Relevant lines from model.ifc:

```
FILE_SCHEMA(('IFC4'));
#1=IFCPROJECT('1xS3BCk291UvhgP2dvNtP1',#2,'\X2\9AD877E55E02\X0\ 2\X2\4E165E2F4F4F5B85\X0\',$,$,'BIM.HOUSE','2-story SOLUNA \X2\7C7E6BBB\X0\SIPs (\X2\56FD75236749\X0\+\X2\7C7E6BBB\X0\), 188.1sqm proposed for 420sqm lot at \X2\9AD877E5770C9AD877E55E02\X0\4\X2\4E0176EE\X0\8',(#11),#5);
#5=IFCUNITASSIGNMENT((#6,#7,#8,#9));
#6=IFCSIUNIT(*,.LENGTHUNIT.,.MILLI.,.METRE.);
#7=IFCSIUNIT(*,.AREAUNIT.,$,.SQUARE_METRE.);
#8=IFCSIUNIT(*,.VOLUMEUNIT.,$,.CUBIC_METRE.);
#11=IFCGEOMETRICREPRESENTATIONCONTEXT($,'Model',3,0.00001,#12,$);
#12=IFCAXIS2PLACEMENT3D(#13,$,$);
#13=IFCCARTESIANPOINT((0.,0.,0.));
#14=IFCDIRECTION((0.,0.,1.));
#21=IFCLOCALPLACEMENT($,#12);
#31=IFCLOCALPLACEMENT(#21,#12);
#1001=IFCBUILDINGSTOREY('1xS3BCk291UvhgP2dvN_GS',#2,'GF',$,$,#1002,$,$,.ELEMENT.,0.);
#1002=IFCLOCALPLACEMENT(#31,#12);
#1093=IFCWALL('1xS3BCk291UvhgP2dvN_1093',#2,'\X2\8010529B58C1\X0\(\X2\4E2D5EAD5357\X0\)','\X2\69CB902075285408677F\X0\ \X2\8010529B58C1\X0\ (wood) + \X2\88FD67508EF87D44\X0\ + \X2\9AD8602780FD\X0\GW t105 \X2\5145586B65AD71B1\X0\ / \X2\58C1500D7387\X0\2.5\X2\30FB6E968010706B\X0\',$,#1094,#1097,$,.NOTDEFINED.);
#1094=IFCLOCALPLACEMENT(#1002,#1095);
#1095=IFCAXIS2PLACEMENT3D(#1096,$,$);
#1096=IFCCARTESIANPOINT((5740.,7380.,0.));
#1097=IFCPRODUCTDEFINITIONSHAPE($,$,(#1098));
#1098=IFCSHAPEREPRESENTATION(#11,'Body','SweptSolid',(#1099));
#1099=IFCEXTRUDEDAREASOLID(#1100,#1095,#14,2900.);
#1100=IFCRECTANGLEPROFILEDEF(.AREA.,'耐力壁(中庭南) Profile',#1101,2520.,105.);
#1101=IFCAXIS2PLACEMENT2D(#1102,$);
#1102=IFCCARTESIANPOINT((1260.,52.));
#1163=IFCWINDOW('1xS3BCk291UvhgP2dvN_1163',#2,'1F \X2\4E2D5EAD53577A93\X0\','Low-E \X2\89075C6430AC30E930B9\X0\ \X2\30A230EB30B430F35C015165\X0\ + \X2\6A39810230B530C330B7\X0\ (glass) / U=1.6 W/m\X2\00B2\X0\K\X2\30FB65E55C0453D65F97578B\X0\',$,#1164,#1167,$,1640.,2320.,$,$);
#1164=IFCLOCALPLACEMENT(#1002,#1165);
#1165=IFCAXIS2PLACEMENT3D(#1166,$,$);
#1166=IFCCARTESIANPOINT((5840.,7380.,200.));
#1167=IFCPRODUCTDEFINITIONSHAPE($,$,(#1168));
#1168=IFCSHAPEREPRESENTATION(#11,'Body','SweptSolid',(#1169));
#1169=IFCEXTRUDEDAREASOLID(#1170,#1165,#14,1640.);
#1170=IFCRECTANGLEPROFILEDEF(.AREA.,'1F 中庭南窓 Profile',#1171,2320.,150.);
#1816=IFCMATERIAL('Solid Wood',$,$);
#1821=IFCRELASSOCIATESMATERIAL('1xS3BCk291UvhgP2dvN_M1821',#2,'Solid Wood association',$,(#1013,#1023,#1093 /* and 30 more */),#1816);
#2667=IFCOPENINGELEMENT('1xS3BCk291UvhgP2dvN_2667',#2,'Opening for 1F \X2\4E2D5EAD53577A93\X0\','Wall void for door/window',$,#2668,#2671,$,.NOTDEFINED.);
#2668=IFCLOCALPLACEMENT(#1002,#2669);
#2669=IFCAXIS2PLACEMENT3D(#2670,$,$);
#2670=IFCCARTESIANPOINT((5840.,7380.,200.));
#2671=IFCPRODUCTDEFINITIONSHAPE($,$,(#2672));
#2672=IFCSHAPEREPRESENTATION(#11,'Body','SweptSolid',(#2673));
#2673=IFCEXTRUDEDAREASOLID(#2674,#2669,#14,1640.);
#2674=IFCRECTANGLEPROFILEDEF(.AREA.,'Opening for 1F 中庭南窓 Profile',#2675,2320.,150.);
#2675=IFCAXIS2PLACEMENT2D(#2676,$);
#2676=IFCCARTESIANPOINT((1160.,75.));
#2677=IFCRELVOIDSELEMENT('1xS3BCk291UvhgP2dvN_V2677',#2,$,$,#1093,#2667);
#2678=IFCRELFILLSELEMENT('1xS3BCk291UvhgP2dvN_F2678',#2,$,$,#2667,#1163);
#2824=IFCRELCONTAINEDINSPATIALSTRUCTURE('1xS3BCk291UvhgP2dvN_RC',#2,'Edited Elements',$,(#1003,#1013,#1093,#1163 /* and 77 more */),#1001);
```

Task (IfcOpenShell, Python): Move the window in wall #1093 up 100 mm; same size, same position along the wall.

```python
import numpy as np
import ifcopenshell
import ifcopenshell.api.geometry
import ifcopenshell.util.placement
import ifcopenshell.util.unit

model = ifcopenshell.open("model.ifc")
unit_scale = ifcopenshell.util.unit.calculate_unit_scale(model)

window = model.by_guid("1xS3BCk291UvhgP2dvN_1163")
opening = window.FillsVoids[0].RelatingOpeningElement
dz = 0.1 / unit_scale

shift = np.array([0.0, 0.0, dz])
# The window is not placed relative to its opening, so move both.
for product in (opening, window):
    matrix = ifcopenshell.util.placement.get_local_placement(product.ObjectPlacement)
    matrix[:3, 3] += shift
    ifcopenshell.api.geometry.edit_object_placement(model, product=product, matrix=matrix, is_si=False)

print(f"moved by {dz * unit_scale:+.3f} m")

model.write("model_rev.ifc")
```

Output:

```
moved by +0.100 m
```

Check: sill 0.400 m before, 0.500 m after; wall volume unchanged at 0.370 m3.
